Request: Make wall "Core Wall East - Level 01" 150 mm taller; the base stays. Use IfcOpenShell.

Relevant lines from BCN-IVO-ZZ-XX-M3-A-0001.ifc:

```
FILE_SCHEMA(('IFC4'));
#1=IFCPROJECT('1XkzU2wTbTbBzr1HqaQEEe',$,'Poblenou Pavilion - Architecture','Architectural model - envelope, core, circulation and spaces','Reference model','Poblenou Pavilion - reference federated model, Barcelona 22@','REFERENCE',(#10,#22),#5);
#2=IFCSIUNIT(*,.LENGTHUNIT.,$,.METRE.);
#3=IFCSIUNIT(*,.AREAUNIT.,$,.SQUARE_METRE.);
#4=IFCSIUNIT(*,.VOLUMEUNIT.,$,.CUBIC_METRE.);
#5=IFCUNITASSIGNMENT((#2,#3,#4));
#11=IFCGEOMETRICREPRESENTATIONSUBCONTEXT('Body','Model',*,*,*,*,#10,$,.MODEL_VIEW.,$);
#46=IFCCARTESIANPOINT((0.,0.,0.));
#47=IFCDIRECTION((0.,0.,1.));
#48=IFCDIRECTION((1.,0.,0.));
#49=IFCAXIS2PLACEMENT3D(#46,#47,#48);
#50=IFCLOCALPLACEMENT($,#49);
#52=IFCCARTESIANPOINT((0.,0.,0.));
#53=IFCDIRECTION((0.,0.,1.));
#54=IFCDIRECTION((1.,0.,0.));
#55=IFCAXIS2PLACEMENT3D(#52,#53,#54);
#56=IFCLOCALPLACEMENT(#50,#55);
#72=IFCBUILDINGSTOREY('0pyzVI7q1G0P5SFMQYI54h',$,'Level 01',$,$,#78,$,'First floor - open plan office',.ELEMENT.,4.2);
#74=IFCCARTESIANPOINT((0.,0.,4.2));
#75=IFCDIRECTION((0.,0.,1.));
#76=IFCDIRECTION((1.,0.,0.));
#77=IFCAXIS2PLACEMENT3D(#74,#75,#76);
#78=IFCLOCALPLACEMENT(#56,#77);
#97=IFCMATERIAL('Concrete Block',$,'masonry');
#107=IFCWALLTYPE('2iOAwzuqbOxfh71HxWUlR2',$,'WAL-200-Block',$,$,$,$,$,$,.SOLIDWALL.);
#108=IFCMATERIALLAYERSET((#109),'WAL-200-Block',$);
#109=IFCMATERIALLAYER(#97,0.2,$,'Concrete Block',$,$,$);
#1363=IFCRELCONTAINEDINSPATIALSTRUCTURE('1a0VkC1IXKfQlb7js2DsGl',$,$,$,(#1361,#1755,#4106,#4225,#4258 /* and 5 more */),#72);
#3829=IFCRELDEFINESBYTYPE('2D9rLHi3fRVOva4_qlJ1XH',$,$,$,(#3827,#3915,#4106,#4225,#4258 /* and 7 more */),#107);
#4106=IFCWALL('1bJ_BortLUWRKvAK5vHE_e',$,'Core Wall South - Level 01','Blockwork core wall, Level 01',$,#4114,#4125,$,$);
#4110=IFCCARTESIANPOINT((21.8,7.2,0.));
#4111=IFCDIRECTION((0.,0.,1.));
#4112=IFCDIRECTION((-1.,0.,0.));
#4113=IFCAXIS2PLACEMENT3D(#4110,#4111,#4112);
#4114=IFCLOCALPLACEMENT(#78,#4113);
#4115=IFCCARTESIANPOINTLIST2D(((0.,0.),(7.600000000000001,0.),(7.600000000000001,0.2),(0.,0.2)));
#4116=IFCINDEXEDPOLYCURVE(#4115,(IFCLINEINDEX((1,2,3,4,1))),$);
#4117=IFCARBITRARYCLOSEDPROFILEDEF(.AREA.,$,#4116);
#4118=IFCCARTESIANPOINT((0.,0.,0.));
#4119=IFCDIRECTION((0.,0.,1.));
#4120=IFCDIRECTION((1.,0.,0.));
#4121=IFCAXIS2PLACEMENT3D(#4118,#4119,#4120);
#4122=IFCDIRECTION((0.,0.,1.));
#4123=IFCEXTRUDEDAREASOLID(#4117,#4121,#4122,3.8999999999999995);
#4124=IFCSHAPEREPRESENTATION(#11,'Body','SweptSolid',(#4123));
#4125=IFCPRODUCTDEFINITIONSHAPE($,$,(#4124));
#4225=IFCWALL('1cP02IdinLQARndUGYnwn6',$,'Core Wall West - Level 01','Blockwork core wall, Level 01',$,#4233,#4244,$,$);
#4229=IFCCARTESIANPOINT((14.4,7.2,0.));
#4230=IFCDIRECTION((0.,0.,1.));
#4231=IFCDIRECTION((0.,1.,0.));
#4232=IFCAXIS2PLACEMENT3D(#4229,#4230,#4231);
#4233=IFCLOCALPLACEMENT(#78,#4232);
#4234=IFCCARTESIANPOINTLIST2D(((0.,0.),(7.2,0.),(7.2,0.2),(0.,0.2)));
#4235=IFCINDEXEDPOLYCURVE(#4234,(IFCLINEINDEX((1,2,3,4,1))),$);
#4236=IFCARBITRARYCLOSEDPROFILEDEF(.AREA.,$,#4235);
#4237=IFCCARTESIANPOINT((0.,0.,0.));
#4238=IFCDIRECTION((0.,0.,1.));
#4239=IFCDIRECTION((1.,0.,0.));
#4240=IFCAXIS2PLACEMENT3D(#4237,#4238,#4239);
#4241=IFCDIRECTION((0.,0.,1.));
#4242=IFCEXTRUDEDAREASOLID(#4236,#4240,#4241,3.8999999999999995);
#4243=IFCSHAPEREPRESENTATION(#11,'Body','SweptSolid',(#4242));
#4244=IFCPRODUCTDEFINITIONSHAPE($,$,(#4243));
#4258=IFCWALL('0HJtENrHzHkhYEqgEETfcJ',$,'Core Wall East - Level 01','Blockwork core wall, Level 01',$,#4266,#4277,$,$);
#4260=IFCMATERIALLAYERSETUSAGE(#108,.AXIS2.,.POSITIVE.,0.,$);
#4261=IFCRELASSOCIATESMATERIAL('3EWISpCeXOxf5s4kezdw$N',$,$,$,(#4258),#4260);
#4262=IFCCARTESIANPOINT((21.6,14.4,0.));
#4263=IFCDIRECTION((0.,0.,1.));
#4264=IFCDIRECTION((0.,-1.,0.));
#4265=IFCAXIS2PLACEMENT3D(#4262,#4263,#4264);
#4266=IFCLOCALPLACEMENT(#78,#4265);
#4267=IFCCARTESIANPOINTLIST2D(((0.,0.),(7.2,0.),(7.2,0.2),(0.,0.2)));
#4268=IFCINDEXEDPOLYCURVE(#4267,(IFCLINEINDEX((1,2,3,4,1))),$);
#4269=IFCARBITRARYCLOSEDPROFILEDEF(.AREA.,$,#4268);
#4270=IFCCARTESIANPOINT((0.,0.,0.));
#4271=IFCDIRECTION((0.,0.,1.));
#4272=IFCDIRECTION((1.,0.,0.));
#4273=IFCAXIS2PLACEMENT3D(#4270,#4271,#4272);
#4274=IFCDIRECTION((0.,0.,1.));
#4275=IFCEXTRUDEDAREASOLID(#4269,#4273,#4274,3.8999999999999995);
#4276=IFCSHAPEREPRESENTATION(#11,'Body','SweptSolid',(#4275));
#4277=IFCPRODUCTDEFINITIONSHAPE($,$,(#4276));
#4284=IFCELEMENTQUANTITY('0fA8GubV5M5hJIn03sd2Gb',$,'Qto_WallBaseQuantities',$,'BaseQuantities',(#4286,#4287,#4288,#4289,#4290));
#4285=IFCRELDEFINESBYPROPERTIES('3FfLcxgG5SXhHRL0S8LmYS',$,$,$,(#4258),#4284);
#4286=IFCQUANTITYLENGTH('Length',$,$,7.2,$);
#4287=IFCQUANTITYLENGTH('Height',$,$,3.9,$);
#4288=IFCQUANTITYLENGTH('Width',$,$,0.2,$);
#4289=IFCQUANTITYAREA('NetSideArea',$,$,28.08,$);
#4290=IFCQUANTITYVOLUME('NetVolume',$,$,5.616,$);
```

```python
import ifcopenshell
import ifcopenshell.api.pset
import ifcopenshell.geom
import ifcopenshell.util.element
import ifcopenshell.util.representation
import ifcopenshell.util.shape
import ifcopenshell.util.unit

model = ifcopenshell.open("BCN-IVO-ZZ-XX-M3-A-0001.ifc")
unit_scale = ifcopenshell.util.unit.calculate_unit_scale(model)
area_scale = ifcopenshell.util.unit.calculate_unit_scale(model, "AREAUNIT")
volume_scale = ifcopenshell.util.unit.calculate_unit_scale(model, "VOLUMEUNIT")
settings = ifcopenshell.geom.settings()


def volume(element):
    """Net volume in cubic metres, openings subtracted."""
    shape = ifcopenshell.geom.create_shape(settings, element)
    return ifcopenshell.util.shape.get_volume(shape.geometry)


wall = model.by_guid("0HJtENrHzHkhYEqgEETfcJ")
before = volume(wall)

body = ifcopenshell.util.representation.get_representation(wall, "Model", "Body")
solid = body.Items[0]
old_height = solid.Depth
solid.Depth += 0.15 / unit_scale
after = volume(wall)
thickness = 0.2  # wall thickness in metres

# Update the stored height, areas and volumes.
qto = model.by_id(ifcopenshell.util.element.get_pset(wall, "Qto_WallBaseQuantities", should_inherit=False)["id"])
ifcopenshell.api.pset.edit_qto(model, qto=qto, properties={
    "Height": solid.Depth,
    "NetSideArea": after / thickness / area_scale,
    "NetVolume": after / volume_scale,
})

print(f"height {old_height:g} -> {solid.Depth:g}, volume {before:.3f} -> {after:.3f} m3")

model.write("BCN-IVO-ZZ-XX-M3-A-0001_updated.ifc")
```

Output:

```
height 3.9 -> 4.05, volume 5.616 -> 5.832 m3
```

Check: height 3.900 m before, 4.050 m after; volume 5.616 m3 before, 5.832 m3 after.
